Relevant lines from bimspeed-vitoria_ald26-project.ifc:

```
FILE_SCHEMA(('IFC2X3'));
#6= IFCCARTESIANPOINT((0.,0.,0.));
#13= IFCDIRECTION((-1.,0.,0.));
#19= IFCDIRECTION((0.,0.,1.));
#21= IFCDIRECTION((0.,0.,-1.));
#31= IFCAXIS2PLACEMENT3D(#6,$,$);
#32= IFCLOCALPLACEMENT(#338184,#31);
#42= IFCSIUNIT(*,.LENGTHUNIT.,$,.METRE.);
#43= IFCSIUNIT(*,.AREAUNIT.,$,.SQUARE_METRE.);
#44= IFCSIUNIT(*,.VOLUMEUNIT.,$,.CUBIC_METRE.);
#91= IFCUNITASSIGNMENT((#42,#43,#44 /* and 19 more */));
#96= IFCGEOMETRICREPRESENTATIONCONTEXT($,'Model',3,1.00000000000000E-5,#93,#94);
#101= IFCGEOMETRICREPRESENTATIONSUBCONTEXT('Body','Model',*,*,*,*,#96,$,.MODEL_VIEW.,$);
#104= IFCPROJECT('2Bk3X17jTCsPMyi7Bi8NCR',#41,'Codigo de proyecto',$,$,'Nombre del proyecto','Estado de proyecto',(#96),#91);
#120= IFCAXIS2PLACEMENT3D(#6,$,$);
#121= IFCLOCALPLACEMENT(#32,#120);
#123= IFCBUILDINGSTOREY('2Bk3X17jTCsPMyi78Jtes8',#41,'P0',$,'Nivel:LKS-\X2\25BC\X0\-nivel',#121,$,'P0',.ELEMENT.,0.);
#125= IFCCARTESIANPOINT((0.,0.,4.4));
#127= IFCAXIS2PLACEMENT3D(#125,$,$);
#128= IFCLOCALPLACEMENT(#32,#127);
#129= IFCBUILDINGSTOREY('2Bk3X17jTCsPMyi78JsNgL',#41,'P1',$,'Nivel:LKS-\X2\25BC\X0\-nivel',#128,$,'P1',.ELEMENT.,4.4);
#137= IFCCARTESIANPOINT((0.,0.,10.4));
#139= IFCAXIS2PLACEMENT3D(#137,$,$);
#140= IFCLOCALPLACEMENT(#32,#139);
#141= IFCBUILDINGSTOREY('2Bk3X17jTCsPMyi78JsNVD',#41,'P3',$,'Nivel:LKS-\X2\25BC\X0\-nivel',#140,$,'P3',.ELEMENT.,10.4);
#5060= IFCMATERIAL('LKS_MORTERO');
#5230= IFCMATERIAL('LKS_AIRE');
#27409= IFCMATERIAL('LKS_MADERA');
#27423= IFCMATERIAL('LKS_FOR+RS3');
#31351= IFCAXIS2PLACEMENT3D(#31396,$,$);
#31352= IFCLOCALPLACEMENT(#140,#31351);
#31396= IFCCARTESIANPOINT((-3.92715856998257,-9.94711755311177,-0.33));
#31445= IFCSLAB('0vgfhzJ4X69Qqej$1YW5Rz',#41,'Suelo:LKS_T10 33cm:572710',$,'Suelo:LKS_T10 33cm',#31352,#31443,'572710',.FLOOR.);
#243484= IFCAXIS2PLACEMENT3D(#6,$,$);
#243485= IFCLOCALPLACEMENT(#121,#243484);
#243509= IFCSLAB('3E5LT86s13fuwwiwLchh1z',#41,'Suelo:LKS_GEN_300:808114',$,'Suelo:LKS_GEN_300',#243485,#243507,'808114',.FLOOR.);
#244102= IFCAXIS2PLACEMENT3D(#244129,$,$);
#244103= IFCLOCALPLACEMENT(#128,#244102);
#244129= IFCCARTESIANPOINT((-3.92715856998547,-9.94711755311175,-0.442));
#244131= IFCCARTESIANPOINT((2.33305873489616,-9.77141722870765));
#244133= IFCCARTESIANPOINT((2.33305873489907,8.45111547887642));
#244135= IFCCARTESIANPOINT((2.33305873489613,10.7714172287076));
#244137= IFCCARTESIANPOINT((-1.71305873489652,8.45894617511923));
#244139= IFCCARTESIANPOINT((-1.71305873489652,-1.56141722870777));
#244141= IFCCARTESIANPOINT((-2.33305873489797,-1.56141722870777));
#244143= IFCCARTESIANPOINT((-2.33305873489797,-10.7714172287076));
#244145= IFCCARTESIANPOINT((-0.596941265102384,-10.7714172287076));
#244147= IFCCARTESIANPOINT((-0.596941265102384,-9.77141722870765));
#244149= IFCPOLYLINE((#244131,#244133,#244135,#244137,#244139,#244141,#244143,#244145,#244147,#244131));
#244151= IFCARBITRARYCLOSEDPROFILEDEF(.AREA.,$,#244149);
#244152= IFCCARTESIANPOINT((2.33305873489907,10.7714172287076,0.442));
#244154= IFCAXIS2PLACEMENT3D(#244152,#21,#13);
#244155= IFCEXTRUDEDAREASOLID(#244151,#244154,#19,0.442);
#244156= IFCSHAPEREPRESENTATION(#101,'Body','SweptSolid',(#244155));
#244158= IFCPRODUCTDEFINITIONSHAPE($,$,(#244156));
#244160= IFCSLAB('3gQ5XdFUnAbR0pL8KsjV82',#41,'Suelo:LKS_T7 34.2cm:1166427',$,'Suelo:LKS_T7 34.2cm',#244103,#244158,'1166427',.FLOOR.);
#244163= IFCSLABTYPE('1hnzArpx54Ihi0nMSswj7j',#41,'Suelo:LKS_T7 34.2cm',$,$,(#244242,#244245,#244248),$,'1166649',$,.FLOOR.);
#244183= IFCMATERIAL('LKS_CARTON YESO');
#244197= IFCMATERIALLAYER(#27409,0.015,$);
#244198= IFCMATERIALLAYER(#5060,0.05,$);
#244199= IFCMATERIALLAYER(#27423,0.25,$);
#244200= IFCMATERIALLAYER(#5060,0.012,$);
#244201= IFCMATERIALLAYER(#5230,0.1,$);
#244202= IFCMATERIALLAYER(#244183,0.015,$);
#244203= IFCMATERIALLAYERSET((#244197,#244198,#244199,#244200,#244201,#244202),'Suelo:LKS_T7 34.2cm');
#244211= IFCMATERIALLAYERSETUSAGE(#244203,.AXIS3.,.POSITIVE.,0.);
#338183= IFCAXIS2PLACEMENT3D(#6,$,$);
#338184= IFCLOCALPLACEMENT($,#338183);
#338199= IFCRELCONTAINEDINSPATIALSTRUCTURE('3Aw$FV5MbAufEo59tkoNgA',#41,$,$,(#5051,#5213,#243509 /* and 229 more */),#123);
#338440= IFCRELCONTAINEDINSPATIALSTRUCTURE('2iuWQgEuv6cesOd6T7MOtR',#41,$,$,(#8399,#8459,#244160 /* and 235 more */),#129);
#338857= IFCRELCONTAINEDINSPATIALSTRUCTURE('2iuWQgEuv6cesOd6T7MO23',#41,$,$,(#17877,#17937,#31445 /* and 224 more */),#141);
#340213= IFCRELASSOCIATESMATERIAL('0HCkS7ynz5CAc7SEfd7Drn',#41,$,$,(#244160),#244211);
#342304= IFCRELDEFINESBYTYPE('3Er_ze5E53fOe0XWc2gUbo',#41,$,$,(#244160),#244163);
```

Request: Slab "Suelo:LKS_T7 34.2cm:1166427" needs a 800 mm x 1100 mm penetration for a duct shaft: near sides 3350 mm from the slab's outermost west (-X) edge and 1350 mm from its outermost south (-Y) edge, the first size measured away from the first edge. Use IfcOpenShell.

```python
import numpy as np
import ifcopenshell
import ifcopenshell.api.feature
import ifcopenshell.api.geometry
import ifcopenshell.api.root
import ifcopenshell.geom
import ifcopenshell.util.placement
import ifcopenshell.util.representation
import ifcopenshell.util.shape
import ifcopenshell.util.unit

model = ifcopenshell.open("bimspeed-vitoria_ald26-project.ifc")
unit_scale = ifcopenshell.util.unit.calculate_unit_scale(model)
settings = ifcopenshell.geom.settings()


def volume(element):
    """Net volume in cubic metres, openings subtracted."""
    shape = ifcopenshell.geom.create_shape(settings, element)
    return ifcopenshell.util.shape.get_volume(shape.geometry)


slab = model.by_guid("3gQ5XdFUnAbR0pL8KsjV82")
before = volume(slab)

# Extent in the slab's own axes, in metres. The edges named are its -X and -Y sides.
slab_shape = ifcopenshell.geom.create_shape(settings, slab)
vertices = ifcopenshell.util.shape.get_vertices(slab_shape.geometry)
x_min, y_min, bottom = vertices.min(axis=0)
top = vertices[:, 2].max()

opening = ifcopenshell.api.root.create_entity(model, ifc_class="IfcOpeningElement", name="Duct shaft opening")
context = ifcopenshell.util.representation.get_context(model, "Model", "Body", "MODEL_VIEW")
width, depth = 0.8, 1.1
outline = [(0.0, 0.0), (width, 0.0), (width, depth), (0.0, depth), (0.0, 0.0)]
# Overshoot both faces by 50 mm so the cut is clean.
shape = ifcopenshell.api.geometry.add_slab_representation(
    model, context=context, depth=top - bottom + 0.1, polyline=outline
)
ifcopenshell.api.geometry.assign_representation(model, product=opening, representation=shape)

matrix = ifcopenshell.util.placement.get_local_placement(slab.ObjectPlacement)
matrix[:, 3] = matrix @ np.append(np.array([x_min + 3.35, y_min + 1.35, bottom - 0.05]) / unit_scale, 1.0)
ifcopenshell.api.geometry.edit_object_placement(model, product=opening, matrix=matrix, is_si=False)
ifcopenshell.api.feature.add_feature(model, feature=opening, element=slab)

after = volume(slab)

print(f"slab volume {before:.3f} -> {after:.3f} m3")

model.write("bimspeed-vitoria_ald26-project_v2.ifc")
```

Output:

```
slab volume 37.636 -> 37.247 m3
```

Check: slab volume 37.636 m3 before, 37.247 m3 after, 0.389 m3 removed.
